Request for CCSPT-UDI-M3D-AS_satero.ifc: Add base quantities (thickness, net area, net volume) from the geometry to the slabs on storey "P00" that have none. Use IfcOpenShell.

First a look at what the model holds.

```python
import ifcopenshell
import ifcopenshell.util.element
import ifcopenshell.util.unit

model = ifcopenshell.open("CCSPT-UDI-M3D-AS_satero.ifc")
print(model.schema)
for unit_type in ("LENGTHUNIT", "AREAUNIT", "VOLUMEUNIT"):
    print(unit_type, ifcopenshell.util.unit.calculate_unit_scale(model, unit_type))
storey = next(s for s in model.by_type("IfcBuildingStorey") if s.Name == "P00")
slabs = [e for e in ifcopenshell.util.element.get_decomposition(storey) if e.is_a("IfcSlab")]
for e in sorted(slabs, key=lambda e: e.id()):
    print(e.id(), e.is_a(), e.Name, list(ifcopenshell.util.element.get_psets(e, qtos_only=True)), sep=" | ")
```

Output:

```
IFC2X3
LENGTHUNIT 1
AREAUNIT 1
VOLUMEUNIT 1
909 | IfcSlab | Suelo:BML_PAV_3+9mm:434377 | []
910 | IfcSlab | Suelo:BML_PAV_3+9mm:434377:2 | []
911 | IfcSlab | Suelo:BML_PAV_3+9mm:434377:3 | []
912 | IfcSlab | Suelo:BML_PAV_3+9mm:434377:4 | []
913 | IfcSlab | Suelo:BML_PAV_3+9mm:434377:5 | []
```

```python
import ifcopenshell
import ifcopenshell.api.pset
import ifcopenshell.geom
import ifcopenshell.util.element
import ifcopenshell.util.shape
import ifcopenshell.util.unit

model = ifcopenshell.open("CCSPT-UDI-M3D-AS_satero.ifc")
unit_scale = ifcopenshell.util.unit.calculate_unit_scale(model)
area_scale = ifcopenshell.util.unit.calculate_unit_scale(model, "AREAUNIT")
volume_scale = ifcopenshell.util.unit.calculate_unit_scale(model, "VOLUMEUNIT")
settings = ifcopenshell.geom.settings()

storey = next(s for s in model.by_type("IfcBuildingStorey") if s.Name == "P00")
slabs = [e for e in ifcopenshell.util.element.get_decomposition(storey) if e.is_a("IfcSlab")]

for e in sorted(slabs, key=lambda e: e.id()):
    if ifcopenshell.util.element.get_psets(e, qtos_only=True, should_inherit=False):
        continue
    # Geometry comes back in metres, in the element's own axes.
    shape = ifcopenshell.geom.create_shape(settings, e)
    values = {
        "Width": ifcopenshell.util.shape.get_z(shape.geometry) / unit_scale,
        "NetArea": ifcopenshell.util.shape.get_footprint_area(shape.geometry) / area_scale,
        "NetVolume": ifcopenshell.util.shape.get_volume(shape.geometry) / volume_scale,
    }
    qto = ifcopenshell.api.pset.add_qto(model, product=e, name="BaseQuantities")
    ifcopenshell.api.pset.edit_qto(model, qto=qto, properties=values)
    print(e.id(), {k: round(v, 3) for k, v in values.items()})

model.write("CCSPT-UDI-M3D-AS_satero_edited.ifc")
```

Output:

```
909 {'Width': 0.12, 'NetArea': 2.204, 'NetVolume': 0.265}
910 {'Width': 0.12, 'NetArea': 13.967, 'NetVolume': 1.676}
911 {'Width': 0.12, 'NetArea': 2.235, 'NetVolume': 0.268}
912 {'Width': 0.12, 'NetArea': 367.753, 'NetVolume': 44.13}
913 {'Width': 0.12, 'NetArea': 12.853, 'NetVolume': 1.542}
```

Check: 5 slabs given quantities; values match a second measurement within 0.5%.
